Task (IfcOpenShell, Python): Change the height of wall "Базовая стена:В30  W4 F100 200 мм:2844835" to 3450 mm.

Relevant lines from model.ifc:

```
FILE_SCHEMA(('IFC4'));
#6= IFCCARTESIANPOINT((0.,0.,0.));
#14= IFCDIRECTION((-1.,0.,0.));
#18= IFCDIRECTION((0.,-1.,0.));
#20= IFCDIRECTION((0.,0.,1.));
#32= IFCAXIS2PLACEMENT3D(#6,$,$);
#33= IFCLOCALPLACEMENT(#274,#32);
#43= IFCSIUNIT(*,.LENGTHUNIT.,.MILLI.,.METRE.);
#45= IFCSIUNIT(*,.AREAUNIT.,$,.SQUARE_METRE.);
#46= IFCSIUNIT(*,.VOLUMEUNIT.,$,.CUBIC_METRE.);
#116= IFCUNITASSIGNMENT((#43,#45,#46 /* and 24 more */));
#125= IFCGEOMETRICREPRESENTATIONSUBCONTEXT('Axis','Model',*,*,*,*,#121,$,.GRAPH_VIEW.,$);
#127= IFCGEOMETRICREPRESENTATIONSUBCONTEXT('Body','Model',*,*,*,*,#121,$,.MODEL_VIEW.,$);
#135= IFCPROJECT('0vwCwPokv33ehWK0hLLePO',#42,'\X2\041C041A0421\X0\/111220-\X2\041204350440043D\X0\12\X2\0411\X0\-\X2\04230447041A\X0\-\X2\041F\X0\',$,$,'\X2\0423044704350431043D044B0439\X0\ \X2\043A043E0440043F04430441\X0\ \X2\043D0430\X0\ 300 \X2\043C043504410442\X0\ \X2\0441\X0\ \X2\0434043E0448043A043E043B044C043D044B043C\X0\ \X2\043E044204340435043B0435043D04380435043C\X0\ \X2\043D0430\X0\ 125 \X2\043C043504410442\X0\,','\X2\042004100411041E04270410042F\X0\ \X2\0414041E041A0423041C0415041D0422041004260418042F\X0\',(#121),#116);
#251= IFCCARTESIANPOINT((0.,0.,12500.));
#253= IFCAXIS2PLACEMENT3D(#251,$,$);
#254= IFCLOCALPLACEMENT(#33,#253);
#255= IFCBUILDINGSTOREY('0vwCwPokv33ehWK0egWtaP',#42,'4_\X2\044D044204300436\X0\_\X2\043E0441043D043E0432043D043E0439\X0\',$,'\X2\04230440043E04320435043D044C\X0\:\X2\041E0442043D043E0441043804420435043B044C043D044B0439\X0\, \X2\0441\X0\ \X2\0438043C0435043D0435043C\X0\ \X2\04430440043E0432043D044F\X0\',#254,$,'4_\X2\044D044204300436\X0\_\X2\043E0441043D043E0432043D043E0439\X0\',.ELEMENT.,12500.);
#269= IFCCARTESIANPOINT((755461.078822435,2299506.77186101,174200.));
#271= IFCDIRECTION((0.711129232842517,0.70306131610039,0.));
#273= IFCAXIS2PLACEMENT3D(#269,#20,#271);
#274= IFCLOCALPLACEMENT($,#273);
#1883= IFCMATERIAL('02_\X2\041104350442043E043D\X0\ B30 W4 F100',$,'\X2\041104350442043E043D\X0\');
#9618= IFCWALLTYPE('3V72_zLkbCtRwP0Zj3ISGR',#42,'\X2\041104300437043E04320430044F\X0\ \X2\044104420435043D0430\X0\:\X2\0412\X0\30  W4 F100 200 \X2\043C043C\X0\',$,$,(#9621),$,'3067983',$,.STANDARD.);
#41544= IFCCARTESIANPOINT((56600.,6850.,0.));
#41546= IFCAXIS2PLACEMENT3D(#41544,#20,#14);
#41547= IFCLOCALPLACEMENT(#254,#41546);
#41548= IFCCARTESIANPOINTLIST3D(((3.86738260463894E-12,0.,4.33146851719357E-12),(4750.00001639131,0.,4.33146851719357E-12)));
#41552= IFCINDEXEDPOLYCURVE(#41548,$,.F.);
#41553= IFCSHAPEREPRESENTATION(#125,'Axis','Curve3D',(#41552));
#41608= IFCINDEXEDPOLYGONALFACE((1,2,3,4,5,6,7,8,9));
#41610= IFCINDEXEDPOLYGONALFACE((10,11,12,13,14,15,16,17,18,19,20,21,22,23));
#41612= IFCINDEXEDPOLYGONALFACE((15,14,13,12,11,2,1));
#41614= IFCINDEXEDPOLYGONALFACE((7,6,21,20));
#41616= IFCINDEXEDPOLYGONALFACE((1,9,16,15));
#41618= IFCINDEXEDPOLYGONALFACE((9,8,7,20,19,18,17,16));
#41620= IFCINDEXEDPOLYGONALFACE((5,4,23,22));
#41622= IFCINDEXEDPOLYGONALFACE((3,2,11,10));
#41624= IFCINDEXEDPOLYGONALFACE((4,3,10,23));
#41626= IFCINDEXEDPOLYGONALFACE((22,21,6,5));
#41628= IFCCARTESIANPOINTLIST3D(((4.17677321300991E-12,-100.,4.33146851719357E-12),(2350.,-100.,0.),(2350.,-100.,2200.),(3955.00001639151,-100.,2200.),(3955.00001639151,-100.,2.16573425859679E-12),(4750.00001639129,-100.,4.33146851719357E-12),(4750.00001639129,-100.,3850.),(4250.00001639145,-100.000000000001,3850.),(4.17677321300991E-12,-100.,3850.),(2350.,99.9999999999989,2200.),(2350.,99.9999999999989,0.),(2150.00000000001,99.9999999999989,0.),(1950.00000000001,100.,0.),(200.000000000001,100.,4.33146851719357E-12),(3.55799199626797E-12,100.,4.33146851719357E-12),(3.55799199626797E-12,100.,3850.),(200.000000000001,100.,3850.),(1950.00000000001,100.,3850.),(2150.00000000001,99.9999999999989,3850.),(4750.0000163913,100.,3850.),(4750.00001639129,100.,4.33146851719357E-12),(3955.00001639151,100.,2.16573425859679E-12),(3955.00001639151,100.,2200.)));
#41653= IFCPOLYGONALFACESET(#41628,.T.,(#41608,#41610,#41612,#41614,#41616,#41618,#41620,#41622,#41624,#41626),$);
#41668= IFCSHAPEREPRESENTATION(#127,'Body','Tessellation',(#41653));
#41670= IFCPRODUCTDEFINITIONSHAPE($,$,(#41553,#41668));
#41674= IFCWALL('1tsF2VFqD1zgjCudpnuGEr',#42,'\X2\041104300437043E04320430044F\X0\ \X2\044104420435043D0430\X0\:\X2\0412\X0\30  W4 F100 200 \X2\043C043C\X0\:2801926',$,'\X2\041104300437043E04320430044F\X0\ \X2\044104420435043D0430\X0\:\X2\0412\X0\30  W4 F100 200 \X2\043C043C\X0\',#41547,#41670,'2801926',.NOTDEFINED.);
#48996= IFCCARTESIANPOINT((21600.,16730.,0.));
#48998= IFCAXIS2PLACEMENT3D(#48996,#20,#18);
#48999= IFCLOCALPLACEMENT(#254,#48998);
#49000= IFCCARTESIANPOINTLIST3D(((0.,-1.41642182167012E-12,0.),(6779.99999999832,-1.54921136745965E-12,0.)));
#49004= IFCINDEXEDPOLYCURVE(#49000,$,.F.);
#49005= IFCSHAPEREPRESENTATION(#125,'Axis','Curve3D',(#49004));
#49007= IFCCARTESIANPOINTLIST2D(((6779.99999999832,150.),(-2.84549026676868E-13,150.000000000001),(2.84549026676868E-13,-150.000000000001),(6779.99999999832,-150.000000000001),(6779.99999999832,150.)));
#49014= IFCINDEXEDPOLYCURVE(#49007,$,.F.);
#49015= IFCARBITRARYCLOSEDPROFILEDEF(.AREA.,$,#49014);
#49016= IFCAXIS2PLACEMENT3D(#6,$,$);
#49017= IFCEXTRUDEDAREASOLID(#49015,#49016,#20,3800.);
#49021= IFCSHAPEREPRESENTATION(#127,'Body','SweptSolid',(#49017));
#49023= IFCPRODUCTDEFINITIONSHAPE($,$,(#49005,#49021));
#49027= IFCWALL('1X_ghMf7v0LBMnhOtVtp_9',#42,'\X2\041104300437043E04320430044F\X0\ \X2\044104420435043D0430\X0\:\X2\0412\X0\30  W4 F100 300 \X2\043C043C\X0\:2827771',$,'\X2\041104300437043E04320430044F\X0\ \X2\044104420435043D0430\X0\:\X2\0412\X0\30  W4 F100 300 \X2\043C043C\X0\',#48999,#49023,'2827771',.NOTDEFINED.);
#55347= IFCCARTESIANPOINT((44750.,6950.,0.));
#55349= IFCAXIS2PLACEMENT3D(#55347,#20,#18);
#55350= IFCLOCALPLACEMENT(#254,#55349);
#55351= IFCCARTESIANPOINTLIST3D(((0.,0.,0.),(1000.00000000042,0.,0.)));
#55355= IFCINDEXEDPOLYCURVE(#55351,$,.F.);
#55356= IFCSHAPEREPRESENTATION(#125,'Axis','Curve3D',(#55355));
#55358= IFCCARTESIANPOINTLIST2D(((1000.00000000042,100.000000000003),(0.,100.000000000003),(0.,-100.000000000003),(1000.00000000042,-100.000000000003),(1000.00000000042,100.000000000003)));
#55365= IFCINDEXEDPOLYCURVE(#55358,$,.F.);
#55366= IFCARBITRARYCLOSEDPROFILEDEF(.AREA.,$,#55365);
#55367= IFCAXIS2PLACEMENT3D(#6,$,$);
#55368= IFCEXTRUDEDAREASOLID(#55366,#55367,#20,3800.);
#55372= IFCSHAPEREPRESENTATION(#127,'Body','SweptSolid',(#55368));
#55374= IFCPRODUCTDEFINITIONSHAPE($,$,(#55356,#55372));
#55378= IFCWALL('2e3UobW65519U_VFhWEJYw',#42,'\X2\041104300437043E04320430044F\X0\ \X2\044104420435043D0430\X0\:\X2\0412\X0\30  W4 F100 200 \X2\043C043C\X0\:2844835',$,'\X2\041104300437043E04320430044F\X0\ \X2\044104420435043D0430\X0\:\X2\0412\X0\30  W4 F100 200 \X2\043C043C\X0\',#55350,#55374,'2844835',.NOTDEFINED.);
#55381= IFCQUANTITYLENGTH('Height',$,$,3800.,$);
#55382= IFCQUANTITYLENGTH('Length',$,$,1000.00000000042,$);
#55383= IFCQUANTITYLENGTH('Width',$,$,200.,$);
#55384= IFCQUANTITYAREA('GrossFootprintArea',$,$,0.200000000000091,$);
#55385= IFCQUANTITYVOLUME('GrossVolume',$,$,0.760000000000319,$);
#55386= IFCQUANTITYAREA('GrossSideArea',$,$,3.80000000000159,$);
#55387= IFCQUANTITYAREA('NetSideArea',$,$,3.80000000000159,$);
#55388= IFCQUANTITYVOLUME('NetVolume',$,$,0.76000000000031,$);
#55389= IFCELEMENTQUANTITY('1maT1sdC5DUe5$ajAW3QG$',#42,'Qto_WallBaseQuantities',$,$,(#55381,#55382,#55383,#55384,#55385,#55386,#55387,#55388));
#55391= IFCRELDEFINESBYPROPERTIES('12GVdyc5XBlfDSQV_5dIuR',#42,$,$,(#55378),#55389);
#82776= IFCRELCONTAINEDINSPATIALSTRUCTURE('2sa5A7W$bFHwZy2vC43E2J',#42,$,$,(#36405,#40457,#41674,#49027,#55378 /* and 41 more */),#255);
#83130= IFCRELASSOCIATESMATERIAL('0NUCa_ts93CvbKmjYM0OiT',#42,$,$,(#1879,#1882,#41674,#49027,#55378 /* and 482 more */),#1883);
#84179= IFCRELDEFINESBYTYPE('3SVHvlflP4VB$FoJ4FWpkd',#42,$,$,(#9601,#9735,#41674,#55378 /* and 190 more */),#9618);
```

```python
import ifcopenshell
import ifcopenshell.api.pset
import ifcopenshell.geom
import ifcopenshell.util.element
import ifcopenshell.util.representation
import ifcopenshell.util.shape
import ifcopenshell.util.unit

model = ifcopenshell.open("model.ifc")
unit_scale = ifcopenshell.util.unit.calculate_unit_scale(model)
area_scale = ifcopenshell.util.unit.calculate_unit_scale(model, "AREAUNIT")
volume_scale = ifcopenshell.util.unit.calculate_unit_scale(model, "VOLUMEUNIT")
settings = ifcopenshell.geom.settings()


def volume(element):
    """Net volume in cubic metres, openings subtracted."""
    shape = ifcopenshell.geom.create_shape(settings, element)
    return ifcopenshell.util.shape.get_volume(shape.geometry)


wall = model.by_id(55378)
before = volume(wall)

body = ifcopenshell.util.representation.get_representation(wall, "Model", "Body")
solid = body.Items[0]
old_height = solid.Depth
solid.Depth = 3.45 / unit_scale
after = volume(wall)
thickness = 0.2  # wall thickness in metres

# Update the stored height, areas and volumes.
qto = model.by_id(ifcopenshell.util.element.get_pset(wall, "Qto_WallBaseQuantities", should_inherit=False)["id"])
ifcopenshell.api.pset.edit_qto(model, qto=qto, properties={
    "Height": solid.Depth,
    "GrossVolume": ifcopenshell.util.element.get_pset(wall, "Qto_WallBaseQuantities", "GrossVolume") * solid.Depth / old_height,
    "GrossSideArea": ifcopenshell.util.element.get_pset(wall, "Qto_WallBaseQuantities", "GrossSideArea") * solid.Depth / old_height,
    "NetSideArea": after / thickness / area_scale,
    "NetVolume": after / volume_scale,
})

print(f"height {old_height:g} -> {solid.Depth:g}, volume {before:.3f} -> {after:.3f} m3")

model.write("model_v2.ifc")
```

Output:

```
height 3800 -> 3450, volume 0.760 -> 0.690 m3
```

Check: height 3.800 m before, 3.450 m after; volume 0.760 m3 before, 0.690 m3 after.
